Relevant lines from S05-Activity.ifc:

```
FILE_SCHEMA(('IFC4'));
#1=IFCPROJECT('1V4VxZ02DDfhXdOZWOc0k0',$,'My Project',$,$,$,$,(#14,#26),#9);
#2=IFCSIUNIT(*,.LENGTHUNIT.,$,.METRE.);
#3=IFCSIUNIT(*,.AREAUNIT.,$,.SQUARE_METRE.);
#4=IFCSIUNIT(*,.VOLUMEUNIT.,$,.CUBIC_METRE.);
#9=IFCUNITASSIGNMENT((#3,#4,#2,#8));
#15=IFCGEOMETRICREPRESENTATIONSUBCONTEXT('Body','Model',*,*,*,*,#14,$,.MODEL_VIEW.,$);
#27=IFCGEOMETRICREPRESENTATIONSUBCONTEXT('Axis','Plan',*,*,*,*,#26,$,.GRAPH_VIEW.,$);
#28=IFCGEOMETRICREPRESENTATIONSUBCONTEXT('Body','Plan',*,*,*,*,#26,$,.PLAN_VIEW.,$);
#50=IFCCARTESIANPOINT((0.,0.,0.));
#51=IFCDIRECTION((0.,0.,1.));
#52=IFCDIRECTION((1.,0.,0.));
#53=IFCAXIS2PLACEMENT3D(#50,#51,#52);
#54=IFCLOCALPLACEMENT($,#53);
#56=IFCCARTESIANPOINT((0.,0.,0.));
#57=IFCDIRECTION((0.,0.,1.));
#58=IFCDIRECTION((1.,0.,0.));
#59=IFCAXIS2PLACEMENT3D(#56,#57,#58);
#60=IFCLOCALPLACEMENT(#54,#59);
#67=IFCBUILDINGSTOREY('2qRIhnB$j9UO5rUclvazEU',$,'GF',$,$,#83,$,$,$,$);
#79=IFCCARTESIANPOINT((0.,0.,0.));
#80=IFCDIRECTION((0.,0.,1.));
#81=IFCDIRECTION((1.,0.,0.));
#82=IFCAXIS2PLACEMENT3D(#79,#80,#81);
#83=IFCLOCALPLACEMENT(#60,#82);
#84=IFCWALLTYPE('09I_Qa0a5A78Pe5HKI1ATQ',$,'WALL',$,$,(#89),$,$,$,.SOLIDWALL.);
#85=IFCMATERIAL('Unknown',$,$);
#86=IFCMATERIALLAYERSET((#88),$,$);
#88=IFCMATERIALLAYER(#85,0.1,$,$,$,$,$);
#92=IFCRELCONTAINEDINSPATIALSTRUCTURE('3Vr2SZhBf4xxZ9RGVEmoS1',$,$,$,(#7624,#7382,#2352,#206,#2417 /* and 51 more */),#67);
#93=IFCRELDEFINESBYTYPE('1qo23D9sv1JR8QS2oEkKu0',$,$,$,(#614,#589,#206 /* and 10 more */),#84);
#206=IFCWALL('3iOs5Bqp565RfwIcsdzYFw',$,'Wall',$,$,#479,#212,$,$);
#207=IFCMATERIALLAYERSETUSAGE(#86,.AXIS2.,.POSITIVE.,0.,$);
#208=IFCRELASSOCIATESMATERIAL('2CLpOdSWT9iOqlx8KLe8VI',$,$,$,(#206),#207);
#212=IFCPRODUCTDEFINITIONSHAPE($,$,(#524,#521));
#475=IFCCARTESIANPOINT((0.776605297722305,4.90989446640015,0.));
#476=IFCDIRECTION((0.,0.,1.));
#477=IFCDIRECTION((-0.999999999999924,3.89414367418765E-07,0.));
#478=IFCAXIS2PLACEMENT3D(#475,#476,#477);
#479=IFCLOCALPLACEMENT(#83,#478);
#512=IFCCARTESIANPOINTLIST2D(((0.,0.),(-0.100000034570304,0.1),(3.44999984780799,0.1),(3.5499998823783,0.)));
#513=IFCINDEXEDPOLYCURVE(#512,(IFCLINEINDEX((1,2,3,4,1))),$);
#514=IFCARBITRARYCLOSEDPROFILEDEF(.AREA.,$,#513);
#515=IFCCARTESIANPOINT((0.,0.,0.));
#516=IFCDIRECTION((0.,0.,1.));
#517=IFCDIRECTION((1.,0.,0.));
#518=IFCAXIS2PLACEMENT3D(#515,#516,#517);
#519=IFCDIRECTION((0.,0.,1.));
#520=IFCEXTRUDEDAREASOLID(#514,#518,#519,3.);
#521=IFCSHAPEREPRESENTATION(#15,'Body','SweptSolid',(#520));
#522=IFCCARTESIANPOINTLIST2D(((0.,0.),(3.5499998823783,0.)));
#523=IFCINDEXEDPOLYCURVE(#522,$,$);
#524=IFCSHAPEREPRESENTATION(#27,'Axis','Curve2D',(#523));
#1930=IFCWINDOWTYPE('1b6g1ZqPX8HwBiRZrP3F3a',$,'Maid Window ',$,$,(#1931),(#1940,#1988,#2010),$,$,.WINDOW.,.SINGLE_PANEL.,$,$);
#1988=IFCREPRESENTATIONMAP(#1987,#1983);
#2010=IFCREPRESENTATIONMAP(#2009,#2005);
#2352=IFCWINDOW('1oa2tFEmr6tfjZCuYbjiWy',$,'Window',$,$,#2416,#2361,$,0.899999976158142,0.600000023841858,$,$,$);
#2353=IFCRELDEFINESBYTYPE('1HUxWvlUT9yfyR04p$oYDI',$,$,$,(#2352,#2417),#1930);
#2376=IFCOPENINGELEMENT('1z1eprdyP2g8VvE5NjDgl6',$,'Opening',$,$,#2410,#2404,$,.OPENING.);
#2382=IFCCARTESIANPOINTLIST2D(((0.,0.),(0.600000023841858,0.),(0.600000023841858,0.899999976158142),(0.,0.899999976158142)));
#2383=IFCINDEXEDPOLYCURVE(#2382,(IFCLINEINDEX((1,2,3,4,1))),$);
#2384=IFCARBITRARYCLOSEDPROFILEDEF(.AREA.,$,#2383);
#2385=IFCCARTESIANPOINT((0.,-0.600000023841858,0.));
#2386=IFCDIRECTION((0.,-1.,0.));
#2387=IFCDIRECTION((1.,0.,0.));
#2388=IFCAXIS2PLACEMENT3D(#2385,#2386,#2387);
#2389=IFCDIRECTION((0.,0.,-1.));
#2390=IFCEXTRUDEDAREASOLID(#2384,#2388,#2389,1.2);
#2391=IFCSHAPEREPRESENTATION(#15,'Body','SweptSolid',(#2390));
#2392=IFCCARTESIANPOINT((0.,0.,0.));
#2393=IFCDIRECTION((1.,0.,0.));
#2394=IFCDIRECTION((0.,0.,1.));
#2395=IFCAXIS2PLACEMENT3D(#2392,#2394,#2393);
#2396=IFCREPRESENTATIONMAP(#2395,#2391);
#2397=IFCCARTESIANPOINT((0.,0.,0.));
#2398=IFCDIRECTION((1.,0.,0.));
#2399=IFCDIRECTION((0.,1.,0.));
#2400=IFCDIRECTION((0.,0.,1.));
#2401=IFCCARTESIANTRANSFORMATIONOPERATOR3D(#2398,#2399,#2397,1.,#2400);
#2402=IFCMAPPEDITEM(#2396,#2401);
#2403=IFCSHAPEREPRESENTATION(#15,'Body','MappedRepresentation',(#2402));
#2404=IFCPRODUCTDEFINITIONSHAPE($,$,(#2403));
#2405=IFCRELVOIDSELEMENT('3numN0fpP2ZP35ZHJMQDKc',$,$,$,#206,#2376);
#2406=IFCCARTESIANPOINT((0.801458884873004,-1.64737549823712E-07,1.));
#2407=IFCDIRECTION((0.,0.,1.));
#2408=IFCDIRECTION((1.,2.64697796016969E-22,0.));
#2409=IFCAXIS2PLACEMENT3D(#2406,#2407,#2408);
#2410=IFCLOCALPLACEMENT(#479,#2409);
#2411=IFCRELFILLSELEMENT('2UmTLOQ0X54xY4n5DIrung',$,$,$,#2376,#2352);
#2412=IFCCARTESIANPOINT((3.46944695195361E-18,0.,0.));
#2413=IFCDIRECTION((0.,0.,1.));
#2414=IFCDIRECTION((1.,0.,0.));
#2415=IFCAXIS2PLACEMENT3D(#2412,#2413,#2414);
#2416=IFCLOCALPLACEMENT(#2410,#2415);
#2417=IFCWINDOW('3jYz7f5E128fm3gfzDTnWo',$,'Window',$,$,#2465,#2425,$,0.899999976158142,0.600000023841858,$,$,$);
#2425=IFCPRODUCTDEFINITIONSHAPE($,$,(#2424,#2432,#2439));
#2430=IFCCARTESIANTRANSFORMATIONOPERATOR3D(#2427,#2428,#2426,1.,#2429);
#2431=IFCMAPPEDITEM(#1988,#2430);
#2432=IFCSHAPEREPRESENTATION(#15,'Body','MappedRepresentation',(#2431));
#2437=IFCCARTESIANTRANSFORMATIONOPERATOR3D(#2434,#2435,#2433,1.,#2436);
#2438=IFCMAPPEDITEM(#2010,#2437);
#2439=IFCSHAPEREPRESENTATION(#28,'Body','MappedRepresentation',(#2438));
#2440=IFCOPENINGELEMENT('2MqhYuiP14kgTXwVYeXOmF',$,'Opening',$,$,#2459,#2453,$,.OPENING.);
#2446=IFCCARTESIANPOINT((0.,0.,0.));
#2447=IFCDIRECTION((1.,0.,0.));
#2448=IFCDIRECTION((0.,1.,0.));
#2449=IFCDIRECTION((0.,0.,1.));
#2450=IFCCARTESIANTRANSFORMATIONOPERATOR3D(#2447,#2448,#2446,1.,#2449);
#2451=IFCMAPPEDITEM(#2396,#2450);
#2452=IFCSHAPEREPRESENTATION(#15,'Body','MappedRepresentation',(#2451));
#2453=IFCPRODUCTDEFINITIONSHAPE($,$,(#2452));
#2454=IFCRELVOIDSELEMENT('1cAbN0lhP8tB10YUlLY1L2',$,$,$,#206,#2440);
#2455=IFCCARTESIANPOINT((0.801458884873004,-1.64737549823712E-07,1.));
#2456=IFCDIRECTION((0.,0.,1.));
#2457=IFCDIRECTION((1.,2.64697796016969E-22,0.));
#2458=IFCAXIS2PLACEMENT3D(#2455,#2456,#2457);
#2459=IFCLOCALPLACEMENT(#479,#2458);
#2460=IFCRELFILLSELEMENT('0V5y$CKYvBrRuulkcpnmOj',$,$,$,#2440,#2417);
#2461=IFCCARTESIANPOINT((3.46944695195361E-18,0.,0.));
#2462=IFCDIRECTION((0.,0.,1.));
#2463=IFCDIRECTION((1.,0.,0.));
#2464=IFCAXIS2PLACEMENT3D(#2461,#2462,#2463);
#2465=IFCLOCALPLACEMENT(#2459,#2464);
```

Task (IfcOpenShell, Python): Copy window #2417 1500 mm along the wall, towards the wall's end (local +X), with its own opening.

```python
import ifcopenshell
import ifcopenshell.api.feature
import ifcopenshell.api.geometry
import ifcopenshell.api.root
import ifcopenshell.geom
import ifcopenshell.util.element
import ifcopenshell.util.placement
import ifcopenshell.util.shape

model = ifcopenshell.open("S05-Activity.ifc")
settings = ifcopenshell.geom.settings()


def volume(element):
    """Net volume in cubic metres, openings subtracted."""
    shape = ifcopenshell.geom.create_shape(settings, element)
    return ifcopenshell.util.shape.get_volume(shape.geometry)


window = model.by_id(2417)
opening = window.FillsVoids[0].RelatingOpeningElement
wall = opening.VoidsElements[0].RelatingBuildingElement
before = volume(wall)
shift = ifcopenshell.util.placement.get_local_placement(wall.ObjectPlacement)[:3, 0] * 1.5

# copy_class copies the void relationship, type, container and properties, but no geometry.
new_opening = ifcopenshell.api.root.copy_class(model, product=opening)
new_opening.Representation = ifcopenshell.util.element.copy_deep(
    model, opening.Representation, exclude=["IfcGeometricRepresentationContext", "IfcRepresentationMap"]
)
new_window = ifcopenshell.api.root.copy_class(model, product=window)
new_window.Representation = ifcopenshell.util.element.copy_deep(
    model, window.Representation, exclude=["IfcGeometricRepresentationContext", "IfcRepresentationMap"]
)
ifcopenshell.api.feature.add_filling(model, opening=new_opening, element=new_window)

for old, new in ((opening, new_opening), (window, new_window)):
    matrix = ifcopenshell.util.placement.get_local_placement(old.ObjectPlacement)
    matrix[:3, 3] += shift
    ifcopenshell.api.geometry.edit_object_placement(model, product=new, matrix=matrix, is_si=False)

after = volume(wall)

print(f"wall volume {before:.3f} -> {after:.3f} m3")

model.write("S05-Activity_edited.ifc")
```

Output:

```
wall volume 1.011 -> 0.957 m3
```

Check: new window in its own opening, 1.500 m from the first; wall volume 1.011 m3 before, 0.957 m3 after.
